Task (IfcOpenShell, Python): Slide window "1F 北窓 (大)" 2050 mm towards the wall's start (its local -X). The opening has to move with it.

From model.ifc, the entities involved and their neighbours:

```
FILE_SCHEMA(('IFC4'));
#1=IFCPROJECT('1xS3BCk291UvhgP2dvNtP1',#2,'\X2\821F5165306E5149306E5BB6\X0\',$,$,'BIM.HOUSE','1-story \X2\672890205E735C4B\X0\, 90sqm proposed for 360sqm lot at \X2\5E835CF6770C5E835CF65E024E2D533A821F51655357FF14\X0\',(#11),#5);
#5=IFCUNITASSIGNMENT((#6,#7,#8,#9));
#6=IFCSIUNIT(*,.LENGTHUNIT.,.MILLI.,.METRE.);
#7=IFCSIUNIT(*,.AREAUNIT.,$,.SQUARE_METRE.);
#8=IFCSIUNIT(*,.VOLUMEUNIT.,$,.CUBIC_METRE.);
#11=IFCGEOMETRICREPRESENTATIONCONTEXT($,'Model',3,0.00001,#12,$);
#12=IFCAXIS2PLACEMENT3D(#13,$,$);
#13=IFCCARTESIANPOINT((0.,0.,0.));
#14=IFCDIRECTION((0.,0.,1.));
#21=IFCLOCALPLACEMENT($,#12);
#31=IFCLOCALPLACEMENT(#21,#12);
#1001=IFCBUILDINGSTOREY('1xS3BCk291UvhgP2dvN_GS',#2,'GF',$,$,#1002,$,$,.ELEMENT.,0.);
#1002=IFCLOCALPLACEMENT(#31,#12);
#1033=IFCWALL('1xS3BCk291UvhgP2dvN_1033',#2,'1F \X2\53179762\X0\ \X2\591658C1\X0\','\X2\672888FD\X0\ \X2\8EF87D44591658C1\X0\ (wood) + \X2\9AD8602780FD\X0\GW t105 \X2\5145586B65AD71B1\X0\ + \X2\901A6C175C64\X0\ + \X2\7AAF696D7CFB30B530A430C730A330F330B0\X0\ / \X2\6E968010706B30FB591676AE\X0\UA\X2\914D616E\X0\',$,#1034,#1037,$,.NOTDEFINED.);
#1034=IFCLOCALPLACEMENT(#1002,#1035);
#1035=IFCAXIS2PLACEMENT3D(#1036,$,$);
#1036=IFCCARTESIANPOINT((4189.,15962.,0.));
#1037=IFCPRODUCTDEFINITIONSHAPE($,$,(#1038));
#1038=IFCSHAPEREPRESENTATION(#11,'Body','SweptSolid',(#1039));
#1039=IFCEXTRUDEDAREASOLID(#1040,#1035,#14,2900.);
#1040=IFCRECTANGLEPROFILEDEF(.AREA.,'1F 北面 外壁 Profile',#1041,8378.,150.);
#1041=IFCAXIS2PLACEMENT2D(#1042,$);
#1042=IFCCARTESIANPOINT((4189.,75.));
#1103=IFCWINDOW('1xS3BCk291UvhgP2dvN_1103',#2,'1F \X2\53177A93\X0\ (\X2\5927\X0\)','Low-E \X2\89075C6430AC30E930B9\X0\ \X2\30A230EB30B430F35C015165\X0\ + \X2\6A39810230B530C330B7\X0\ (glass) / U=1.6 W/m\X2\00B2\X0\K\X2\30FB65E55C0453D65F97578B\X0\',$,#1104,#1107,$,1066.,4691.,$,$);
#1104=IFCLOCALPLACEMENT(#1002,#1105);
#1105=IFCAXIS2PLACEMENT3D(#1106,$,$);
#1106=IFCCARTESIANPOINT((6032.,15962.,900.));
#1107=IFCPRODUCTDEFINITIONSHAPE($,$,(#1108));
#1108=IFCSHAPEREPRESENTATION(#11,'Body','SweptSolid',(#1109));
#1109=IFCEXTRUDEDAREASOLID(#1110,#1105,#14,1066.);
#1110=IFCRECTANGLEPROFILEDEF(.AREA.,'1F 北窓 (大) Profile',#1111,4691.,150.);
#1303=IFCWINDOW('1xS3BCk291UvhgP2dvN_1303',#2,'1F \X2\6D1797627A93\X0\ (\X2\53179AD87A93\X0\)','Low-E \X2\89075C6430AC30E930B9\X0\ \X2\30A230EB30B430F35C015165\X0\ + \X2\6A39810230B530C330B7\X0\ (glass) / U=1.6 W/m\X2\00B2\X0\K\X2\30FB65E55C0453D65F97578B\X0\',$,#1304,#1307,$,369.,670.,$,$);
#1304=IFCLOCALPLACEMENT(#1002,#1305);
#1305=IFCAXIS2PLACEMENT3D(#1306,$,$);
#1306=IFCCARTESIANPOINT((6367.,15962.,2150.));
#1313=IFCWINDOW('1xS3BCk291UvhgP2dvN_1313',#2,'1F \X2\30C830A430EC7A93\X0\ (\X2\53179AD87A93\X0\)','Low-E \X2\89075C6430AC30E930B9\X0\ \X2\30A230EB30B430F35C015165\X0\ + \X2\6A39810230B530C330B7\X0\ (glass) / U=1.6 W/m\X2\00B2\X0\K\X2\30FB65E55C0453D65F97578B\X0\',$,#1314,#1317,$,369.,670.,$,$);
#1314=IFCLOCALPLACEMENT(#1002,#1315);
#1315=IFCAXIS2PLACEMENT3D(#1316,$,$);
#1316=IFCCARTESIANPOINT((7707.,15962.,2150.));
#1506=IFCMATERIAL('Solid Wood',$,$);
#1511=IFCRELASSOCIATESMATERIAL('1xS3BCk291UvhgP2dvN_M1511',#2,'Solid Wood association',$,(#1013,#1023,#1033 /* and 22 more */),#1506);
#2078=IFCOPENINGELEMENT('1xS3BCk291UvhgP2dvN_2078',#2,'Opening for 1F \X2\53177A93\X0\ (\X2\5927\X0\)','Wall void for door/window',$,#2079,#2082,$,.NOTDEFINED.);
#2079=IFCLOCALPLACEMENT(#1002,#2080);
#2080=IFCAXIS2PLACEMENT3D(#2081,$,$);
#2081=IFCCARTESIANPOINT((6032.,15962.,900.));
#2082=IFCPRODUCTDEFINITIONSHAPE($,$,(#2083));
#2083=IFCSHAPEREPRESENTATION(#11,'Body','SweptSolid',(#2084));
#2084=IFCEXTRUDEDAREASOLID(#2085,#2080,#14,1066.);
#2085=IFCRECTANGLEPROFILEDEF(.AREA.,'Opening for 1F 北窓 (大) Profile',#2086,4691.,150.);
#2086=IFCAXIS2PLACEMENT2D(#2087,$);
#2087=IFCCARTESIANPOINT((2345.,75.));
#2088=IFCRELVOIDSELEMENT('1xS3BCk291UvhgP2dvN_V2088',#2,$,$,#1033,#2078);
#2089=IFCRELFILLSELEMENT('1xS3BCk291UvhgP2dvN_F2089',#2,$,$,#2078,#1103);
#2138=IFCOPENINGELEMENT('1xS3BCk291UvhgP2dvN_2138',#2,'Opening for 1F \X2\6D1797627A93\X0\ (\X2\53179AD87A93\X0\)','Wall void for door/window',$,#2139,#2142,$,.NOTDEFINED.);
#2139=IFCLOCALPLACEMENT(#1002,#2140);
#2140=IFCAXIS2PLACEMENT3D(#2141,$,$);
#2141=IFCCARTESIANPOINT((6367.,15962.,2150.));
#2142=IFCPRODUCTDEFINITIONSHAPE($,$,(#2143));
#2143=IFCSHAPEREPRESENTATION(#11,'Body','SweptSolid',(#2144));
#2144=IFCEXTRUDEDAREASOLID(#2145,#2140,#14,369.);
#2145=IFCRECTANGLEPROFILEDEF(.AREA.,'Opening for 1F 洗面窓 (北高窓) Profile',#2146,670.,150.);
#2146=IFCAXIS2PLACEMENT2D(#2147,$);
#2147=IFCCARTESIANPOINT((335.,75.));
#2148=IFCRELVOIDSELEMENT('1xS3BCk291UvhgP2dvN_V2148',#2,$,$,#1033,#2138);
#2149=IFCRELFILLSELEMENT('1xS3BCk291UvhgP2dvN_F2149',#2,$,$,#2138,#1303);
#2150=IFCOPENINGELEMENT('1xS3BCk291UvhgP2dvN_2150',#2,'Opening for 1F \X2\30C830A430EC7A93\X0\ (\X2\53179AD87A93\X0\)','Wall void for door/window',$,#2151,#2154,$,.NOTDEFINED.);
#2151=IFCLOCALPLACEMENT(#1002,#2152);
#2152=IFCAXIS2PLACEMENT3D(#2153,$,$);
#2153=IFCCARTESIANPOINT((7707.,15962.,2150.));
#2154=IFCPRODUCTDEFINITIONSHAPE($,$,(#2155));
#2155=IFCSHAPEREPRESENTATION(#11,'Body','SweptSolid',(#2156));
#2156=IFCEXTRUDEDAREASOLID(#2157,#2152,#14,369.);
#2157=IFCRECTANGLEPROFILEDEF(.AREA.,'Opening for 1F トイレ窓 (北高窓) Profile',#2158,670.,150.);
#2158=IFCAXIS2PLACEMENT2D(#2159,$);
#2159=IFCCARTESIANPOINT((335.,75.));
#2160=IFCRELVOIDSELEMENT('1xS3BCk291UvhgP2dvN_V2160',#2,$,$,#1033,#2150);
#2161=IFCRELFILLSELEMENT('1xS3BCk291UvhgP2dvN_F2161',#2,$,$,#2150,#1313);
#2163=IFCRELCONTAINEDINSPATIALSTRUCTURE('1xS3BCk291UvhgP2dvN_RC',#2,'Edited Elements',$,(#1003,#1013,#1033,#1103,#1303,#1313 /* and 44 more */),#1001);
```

```python
import ifcopenshell
import ifcopenshell.api.geometry
import ifcopenshell.util.placement
import ifcopenshell.util.unit

model = ifcopenshell.open("model.ifc")
unit_scale = ifcopenshell.util.unit.calculate_unit_scale(model)

window = model.by_guid("1xS3BCk291UvhgP2dvN_1103")
opening = window.FillsVoids[0].RelatingOpeningElement
wall = opening.VoidsElements[0].RelatingBuildingElement

wall_matrix = ifcopenshell.util.placement.get_local_placement(wall.ObjectPlacement)
shift = wall_matrix[:3, 0] * -2.05 / unit_scale
before = ifcopenshell.util.placement.get_local_placement(window.ObjectPlacement)[:3, 3].copy()

# The window is not placed relative to its opening, so move both.
for product in (opening, window):
    matrix = ifcopenshell.util.placement.get_local_placement(product.ObjectPlacement)
    matrix[:3, 3] += shift
    ifcopenshell.api.geometry.edit_object_placement(model, product=product, matrix=matrix, is_si=False)

after = ifcopenshell.util.placement.get_local_placement(window.ObjectPlacement)[:3, 3]
print("window moved by", (after - before).round(3) + 0.0)

model.write("model_rev.ifc")
```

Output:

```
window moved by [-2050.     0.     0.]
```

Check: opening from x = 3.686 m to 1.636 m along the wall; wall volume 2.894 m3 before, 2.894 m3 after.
